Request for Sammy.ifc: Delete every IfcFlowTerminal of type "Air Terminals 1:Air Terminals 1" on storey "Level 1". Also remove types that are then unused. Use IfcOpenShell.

First a look at what the model holds.

```python
import ifcopenshell
import ifcopenshell.util.element

model = ifcopenshell.open("Sammy.ifc")
print(model.schema)
storey = next(s for s in model.by_type("IfcBuildingStorey") if s.Name == "Level 1")
terminals = [e for e in ifcopenshell.util.element.get_decomposition(storey) if e.is_a("IfcFlowTerminal")]
seen = {}
for e in terminals:
    element_type = ifcopenshell.util.element.get_type(e)
    name = element_type.Name if element_type not in (None, e) else None
    seen[name] = seen.get(name, 0) + 1
for name, count in sorted(seen.items(), key=str):
    print(count, "x", name)
```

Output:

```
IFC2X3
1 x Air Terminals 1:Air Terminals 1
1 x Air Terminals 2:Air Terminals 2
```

```python
import ifcopenshell
import ifcopenshell.api.root
import ifcopenshell.util.element

model = ifcopenshell.open("Sammy.ifc")

storey = next(s for s in model.by_type("IfcBuildingStorey") if s.Name == "Level 1")
terminals = [e for e in ifcopenshell.util.element.get_decomposition(storey) if e.is_a("IfcFlowTerminal")]
targets = [e for e in terminals if (t := ifcopenshell.util.element.get_type(e)) not in (None, e) and t.Name == "Air Terminals 1:Air Terminals 1"]
types = {ifcopenshell.util.element.get_type(e) for e in targets} - {None, *targets}

for e in targets:
    ifcopenshell.api.root.remove_product(model, product=e)
print(len(targets), "removed")

unused = [t for t in types if not ifcopenshell.util.element.get_types(t)]
for t in unused:
    ifcopenshell.api.root.remove_product(model, product=t)
print(len(unused), "unused types removed")

model.write("Sammy_edited.ifc")
```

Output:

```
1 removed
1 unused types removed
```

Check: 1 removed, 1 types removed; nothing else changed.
